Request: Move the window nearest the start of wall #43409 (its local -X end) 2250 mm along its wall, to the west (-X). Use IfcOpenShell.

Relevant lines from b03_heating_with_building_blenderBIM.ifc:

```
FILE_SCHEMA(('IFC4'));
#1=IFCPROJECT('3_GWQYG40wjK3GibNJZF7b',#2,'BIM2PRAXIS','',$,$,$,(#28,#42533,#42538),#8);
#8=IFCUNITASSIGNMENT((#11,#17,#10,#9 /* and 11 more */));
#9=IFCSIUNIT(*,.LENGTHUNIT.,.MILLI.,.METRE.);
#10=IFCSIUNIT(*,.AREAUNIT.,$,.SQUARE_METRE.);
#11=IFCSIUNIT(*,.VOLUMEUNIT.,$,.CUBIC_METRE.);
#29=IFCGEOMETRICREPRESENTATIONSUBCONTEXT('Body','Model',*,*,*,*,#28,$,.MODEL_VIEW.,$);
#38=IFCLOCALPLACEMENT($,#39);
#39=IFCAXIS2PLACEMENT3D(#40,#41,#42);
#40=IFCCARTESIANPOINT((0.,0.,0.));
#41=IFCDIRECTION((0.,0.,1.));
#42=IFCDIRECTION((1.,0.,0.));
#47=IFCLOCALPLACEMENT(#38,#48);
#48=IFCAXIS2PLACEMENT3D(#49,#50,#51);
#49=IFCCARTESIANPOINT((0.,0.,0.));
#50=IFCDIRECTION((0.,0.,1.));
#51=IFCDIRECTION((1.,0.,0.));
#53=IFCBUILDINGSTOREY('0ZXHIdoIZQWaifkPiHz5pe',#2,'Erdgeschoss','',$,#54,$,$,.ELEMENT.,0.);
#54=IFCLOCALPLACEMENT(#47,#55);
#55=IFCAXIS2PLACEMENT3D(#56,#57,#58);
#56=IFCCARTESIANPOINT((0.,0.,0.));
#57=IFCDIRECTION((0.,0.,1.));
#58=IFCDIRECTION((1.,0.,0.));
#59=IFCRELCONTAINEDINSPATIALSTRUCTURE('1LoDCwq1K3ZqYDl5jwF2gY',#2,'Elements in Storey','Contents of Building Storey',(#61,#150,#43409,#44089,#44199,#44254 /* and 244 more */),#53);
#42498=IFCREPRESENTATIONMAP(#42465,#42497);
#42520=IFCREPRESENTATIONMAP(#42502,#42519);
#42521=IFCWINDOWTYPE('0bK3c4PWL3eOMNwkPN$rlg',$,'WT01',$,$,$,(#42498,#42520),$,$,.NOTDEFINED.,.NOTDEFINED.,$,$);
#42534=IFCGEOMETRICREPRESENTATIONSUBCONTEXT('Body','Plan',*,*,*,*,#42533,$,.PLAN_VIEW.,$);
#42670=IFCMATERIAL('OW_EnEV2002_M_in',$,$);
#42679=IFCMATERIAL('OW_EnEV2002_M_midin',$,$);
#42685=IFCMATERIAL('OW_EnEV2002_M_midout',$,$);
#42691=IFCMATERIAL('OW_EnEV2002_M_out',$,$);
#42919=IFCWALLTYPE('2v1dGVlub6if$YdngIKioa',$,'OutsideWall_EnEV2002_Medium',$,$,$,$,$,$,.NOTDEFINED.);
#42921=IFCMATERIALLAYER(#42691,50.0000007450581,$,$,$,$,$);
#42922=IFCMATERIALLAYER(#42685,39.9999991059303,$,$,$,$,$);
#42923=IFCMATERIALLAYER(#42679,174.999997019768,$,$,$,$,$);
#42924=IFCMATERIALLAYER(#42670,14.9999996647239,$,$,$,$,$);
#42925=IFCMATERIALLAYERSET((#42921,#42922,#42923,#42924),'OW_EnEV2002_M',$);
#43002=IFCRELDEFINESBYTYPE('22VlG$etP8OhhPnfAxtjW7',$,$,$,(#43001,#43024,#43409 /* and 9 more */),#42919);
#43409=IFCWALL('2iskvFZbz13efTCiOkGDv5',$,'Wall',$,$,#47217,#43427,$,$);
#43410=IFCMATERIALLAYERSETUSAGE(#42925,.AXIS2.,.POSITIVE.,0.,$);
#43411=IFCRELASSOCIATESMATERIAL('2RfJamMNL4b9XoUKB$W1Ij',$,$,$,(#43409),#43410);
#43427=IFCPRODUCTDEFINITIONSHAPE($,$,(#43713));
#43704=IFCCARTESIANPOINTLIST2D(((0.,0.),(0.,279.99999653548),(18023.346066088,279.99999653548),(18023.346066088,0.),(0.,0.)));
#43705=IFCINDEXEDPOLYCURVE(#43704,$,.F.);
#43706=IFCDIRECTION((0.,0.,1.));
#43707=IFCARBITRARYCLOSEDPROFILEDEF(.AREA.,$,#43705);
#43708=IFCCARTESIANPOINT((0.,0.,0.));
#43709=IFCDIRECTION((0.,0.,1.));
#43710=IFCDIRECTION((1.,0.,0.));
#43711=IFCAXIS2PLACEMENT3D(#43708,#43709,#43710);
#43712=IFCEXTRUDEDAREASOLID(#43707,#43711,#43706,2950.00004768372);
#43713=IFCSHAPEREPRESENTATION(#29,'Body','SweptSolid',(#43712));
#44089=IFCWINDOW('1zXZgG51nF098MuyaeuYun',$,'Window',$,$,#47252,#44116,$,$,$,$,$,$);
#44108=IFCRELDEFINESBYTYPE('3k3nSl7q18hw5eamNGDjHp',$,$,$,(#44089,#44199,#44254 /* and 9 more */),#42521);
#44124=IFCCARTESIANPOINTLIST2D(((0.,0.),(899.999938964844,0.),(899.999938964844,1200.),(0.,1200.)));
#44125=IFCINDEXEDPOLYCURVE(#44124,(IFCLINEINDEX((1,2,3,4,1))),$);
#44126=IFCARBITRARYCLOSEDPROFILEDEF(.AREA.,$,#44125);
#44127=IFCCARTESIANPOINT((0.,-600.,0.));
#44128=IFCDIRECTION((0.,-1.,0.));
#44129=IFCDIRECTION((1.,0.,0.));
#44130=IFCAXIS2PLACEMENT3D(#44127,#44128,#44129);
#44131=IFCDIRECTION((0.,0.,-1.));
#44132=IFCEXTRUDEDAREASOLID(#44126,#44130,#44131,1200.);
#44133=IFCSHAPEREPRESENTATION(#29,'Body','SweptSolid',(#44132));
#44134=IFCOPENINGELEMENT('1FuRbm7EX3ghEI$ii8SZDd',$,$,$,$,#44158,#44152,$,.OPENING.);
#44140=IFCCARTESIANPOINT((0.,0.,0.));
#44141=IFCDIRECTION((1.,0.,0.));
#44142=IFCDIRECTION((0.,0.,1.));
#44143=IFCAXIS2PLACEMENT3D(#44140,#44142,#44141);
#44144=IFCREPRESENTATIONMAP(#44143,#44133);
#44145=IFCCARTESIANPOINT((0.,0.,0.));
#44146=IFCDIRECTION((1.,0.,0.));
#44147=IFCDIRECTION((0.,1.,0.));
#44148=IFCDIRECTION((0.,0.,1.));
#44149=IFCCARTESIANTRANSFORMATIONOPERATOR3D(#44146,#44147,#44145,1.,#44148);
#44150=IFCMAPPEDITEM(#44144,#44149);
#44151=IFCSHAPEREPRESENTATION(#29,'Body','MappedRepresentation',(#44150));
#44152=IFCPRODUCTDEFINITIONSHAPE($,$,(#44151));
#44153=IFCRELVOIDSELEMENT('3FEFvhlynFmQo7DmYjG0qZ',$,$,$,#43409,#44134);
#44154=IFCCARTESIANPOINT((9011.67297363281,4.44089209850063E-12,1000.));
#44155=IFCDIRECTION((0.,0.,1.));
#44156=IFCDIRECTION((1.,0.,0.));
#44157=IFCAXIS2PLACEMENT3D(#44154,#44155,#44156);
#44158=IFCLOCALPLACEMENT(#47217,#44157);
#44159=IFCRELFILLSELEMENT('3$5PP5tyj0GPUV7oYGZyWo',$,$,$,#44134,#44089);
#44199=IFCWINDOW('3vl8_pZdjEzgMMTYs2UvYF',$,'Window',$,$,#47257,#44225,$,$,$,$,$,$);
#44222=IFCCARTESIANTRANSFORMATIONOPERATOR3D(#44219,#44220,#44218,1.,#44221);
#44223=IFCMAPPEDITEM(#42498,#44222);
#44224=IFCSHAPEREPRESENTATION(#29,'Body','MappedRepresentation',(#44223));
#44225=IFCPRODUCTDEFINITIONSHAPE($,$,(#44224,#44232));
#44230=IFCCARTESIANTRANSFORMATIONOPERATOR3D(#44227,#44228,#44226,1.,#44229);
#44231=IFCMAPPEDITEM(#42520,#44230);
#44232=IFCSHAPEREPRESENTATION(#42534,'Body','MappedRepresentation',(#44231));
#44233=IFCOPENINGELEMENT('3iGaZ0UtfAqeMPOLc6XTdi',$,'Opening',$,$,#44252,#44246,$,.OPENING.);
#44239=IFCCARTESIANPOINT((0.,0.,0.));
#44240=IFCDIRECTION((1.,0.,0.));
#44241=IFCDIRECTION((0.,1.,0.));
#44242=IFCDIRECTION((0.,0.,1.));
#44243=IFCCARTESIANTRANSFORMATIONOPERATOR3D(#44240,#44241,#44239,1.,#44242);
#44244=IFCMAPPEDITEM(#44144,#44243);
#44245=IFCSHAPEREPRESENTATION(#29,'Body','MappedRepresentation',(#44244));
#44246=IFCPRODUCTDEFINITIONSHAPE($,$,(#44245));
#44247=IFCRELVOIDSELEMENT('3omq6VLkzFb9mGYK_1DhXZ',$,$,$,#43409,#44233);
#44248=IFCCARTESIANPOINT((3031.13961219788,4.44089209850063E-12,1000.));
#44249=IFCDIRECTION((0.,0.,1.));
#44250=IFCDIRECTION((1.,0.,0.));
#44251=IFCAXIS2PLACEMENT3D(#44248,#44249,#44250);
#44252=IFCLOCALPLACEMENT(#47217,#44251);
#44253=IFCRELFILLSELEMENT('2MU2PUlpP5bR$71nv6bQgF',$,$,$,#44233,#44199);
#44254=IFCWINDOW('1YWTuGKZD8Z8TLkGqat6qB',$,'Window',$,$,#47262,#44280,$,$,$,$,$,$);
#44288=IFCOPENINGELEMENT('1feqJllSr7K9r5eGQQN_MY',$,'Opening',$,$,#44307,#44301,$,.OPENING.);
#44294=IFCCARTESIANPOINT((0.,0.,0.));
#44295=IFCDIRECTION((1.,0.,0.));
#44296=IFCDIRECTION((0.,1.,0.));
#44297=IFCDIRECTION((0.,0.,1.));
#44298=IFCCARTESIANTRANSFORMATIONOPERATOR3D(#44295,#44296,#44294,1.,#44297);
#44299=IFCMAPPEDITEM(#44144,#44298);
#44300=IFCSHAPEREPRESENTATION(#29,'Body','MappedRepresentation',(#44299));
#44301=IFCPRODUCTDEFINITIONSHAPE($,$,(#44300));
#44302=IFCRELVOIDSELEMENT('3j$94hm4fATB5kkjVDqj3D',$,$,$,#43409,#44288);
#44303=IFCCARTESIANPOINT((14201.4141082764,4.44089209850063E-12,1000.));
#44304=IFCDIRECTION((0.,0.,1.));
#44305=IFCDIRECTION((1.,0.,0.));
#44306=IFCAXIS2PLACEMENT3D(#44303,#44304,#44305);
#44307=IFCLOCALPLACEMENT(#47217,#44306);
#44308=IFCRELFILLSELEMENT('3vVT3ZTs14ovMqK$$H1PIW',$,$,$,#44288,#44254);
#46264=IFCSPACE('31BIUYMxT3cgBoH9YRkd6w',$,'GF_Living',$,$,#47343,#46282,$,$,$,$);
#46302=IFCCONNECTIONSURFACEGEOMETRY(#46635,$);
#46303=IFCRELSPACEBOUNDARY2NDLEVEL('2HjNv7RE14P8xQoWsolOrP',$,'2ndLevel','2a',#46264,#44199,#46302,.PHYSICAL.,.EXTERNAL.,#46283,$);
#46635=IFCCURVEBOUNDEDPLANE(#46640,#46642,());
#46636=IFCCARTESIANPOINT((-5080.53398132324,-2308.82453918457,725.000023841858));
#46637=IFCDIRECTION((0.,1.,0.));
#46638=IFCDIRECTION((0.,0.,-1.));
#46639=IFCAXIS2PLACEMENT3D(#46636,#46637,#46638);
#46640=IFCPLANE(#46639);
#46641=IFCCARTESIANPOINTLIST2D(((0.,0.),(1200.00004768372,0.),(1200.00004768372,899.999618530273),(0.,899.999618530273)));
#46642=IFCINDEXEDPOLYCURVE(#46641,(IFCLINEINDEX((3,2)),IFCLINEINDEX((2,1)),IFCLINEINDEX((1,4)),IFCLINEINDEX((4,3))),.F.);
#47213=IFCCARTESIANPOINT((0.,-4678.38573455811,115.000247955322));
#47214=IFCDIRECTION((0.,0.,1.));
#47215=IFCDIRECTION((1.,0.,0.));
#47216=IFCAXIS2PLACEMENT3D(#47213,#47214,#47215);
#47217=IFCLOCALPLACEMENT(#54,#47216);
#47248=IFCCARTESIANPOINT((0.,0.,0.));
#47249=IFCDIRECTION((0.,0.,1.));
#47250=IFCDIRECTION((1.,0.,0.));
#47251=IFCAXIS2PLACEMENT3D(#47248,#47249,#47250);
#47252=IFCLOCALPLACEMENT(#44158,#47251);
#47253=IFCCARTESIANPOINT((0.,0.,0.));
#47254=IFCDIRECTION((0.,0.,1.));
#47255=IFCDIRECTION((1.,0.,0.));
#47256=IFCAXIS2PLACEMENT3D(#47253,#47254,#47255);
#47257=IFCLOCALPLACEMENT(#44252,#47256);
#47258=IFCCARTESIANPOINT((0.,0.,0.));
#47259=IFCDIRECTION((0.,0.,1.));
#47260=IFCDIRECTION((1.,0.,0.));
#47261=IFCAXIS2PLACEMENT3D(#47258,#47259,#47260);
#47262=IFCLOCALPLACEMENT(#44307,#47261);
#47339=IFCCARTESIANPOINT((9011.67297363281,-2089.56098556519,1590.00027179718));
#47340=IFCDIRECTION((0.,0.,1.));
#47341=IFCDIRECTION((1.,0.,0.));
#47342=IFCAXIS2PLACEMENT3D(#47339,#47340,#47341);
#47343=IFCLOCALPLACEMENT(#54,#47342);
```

```python
import numpy as np
import ifcopenshell
import ifcopenshell.api.geometry
import ifcopenshell.util.placement

model = ifcopenshell.open("b03_heating_with_building_blenderBIM.ifc")

window = model.by_guid("3vl8_pZdjEzgMMTYs2UvYF")
opening = window.FillsVoids[0].RelatingOpeningElement
wall = opening.VoidsElements[0].RelatingBuildingElement

wall_matrix = ifcopenshell.util.placement.get_local_placement(wall.ObjectPlacement)
shift = wall_matrix[:3, 0] * -2250.0
before = ifcopenshell.util.placement.get_local_placement(window.ObjectPlacement)[:3, 3].copy()

# The window is placed relative to its opening, so it follows when the opening moves.
matrix = ifcopenshell.util.placement.get_local_placement(opening.ObjectPlacement)
matrix[:3, 3] += shift
ifcopenshell.api.geometry.edit_object_placement(
    model, product=opening, matrix=matrix, is_si=False, should_transform_children=True
)

# Space boundary surfaces are stored in each space's coordinates; move them too.
for rel in window.ProvidesBoundaries:
    if not rel.ConnectionGeometry:
        continue
    surface = rel.ConnectionGeometry.SurfaceOnRelatingElement.BasisSurface
    space_matrix = ifcopenshell.util.placement.get_local_placement(rel.RelatingSpace.ObjectPlacement)
    point = np.array(surface.Position.Location.Coordinates) + space_matrix[:3, :3].T @ shift
    surface.Position = model.createIfcAxis2Placement3D(
        model.createIfcCartesianPoint(point.tolist()), surface.Position.Axis, surface.Position.RefDirection
    )

after = ifcopenshell.util.placement.get_local_placement(window.ObjectPlacement)[:3, 3]
print("window moved by", (after - before).round(3) + 0.0)

model.write("b03_heating_with_building_blenderBIM-out.ifc")
```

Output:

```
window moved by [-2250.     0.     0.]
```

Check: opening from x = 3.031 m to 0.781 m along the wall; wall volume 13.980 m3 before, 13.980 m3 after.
